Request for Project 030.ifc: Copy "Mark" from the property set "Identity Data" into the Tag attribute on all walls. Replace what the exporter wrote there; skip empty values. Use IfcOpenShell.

First a look at what the model holds.

```python
import ifcopenshell
import ifcopenshell.util.element

model = ifcopenshell.open("Project 030.ifc")
print(model.schema)
walls = model.by_type("IfcWall")
print(len(walls), "walls")
for e in walls[:8]:
    source = ifcopenshell.util.element.get_pset(e, "Identity Data", "Mark")
    target = e.Tag
    print(e.id(), repr(source), repr(target), sep=" | ")
```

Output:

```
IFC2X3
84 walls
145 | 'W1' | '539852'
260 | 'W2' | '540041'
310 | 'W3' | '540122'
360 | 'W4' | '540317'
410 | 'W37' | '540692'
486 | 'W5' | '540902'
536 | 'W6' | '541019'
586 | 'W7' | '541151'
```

```python
import ifcopenshell
import ifcopenshell.util.element

model = ifcopenshell.open("Project 030.ifc")

count = 0
for e in model.by_type("IfcWall"):
    value = ifcopenshell.util.element.get_pset(e, "Identity Data", "Mark")
    current = e.Tag
    if not value or not value.strip() or current == value:
        continue
    e.Tag = value
    count += 1

print(count, "walls updated")

model.write("Project 030_rev.ifc")
```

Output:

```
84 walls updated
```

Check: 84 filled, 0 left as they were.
